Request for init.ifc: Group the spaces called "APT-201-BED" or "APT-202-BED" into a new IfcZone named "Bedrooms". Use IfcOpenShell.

First a look at what the model holds.

```python
import ifcopenshell

model = ifcopenshell.open("init.ifc")
print(model.schema)
seen = {}
for space in model.by_type("IfcSpace"):
    seen[space.Name] = seen.get(space.Name, 0) + 1
for name, count in sorted(seen.items(), key=str):
    print(count, "x", name)
print("zones:", [z.Name for z in model.by_type("IfcZone")][:20])
```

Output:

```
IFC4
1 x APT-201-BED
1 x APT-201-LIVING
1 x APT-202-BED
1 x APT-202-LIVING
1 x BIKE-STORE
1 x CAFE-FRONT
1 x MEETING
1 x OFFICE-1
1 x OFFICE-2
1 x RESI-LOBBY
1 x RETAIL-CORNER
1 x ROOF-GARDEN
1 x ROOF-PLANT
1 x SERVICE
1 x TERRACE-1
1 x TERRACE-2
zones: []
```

```python
import ifcopenshell
import ifcopenshell.api.group
import ifcopenshell.api.root

model = ifcopenshell.open("init.ifc")

names = {"APT-201-BED", "APT-202-BED"}
spaces = [s for s in model.by_type("IfcSpace") if s.Name in names]

zone = ifcopenshell.api.root.create_entity(model, ifc_class="IfcZone", name="Bedrooms")
ifcopenshell.api.group.assign_group(model, products=spaces, group=zone)
print(len(spaces), "spaces in", zone.Name)

model.write("init_rev.ifc")
```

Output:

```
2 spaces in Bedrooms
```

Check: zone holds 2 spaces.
